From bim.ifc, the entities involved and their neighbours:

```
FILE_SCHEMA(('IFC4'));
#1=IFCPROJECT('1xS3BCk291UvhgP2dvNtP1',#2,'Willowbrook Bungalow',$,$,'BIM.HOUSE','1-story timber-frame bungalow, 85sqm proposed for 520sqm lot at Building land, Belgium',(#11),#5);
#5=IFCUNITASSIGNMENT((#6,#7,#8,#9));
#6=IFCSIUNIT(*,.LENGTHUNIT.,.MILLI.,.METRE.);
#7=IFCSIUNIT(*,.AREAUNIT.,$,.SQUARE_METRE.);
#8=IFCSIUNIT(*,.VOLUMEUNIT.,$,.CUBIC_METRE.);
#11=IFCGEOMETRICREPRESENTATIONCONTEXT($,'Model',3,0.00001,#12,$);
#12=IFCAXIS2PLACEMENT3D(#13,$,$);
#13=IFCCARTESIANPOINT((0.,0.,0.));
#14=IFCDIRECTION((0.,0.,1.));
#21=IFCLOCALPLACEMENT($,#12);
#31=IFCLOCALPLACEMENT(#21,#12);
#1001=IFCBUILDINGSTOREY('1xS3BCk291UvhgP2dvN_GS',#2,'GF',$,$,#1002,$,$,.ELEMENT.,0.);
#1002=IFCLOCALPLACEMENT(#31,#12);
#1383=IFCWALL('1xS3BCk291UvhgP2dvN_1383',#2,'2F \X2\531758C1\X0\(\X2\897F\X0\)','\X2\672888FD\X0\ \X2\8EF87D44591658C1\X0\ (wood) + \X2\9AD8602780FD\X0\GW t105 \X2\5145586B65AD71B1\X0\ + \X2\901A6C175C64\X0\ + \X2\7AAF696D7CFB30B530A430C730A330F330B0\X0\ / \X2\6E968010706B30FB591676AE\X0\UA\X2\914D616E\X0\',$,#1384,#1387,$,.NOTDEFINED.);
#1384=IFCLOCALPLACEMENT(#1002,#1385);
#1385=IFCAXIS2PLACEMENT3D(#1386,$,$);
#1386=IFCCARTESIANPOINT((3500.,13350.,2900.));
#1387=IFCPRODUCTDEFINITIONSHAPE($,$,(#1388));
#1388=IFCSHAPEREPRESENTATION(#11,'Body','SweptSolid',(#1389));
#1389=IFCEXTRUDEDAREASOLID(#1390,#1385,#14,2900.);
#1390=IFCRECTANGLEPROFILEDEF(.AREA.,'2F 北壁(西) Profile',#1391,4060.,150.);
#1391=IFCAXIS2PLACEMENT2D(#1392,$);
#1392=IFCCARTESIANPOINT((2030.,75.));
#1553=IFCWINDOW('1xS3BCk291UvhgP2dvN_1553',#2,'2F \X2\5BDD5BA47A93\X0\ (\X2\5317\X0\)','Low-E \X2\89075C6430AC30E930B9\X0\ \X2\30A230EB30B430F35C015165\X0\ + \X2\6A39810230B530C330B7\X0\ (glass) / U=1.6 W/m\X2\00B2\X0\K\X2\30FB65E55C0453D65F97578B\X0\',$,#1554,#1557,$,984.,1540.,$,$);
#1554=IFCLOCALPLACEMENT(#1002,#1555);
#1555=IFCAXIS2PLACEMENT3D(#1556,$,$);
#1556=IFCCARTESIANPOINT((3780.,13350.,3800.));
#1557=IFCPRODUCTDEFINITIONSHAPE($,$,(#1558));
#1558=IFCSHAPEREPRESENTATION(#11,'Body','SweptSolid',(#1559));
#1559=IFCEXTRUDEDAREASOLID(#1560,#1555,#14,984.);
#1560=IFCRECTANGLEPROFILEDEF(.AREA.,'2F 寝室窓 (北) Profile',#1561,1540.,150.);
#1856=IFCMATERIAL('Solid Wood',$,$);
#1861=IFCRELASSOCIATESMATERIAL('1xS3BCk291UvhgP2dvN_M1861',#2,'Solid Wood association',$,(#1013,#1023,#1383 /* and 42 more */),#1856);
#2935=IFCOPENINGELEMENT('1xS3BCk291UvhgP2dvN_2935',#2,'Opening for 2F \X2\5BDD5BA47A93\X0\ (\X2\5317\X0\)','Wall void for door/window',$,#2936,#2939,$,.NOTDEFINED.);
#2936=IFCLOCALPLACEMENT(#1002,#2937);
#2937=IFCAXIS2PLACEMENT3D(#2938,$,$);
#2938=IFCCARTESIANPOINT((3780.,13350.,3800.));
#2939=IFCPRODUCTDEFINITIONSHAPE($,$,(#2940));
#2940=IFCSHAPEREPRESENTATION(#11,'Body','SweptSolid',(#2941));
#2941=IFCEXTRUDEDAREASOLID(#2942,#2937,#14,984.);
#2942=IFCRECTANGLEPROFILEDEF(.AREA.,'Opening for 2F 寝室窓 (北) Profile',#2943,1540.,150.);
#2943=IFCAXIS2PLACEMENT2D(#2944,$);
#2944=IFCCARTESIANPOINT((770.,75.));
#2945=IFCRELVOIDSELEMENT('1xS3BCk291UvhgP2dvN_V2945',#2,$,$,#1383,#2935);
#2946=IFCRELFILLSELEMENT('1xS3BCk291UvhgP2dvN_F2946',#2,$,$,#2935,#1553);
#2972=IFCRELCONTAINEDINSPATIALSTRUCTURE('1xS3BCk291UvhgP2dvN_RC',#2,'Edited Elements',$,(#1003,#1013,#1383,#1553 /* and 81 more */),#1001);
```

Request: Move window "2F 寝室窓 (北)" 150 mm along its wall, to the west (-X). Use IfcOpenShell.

```python
import ifcopenshell
import ifcopenshell.api.geometry
import ifcopenshell.util.placement

model = ifcopenshell.open("bim.ifc")

window = model.by_id(1553)
opening = window.FillsVoids[0].RelatingOpeningElement
wall = opening.VoidsElements[0].RelatingBuildingElement

wall_matrix = ifcopenshell.util.placement.get_local_placement(wall.ObjectPlacement)
shift = wall_matrix[:3, 0] * -150.0
before = ifcopenshell.util.placement.get_local_placement(window.ObjectPlacement)[:3, 3].copy()

# The window is not placed relative to its opening, so move both.
for product in (opening, window):
    matrix = ifcopenshell.util.placement.get_local_placement(product.ObjectPlacement)
    matrix[:3, 3] += shift
    ifcopenshell.api.geometry.edit_object_placement(model, product=product, matrix=matrix, is_si=False)

after = ifcopenshell.util.placement.get_local_placement(window.ObjectPlacement)[:3, 3]
print("window moved by", (after - before).round(3) + 0.0)

model.write("bim-out.ifc")
```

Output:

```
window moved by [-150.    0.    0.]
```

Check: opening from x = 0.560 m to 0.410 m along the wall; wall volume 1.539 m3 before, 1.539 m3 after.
